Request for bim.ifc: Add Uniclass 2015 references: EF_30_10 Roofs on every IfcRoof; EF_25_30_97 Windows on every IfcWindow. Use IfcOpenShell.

First a look at what the model holds.

```python
import ifcopenshell

model = ifcopenshell.open("bim.ifc")
print(model.schema)
print("classifications:", [c.Name for c in model.by_type("IfcClassification")])
for ifc_class in ("IfcDoor", "IfcRoof", "IfcStair", "IfcWall", "IfcWindow"):
    print(ifc_class, len(model.by_type(ifc_class)))
```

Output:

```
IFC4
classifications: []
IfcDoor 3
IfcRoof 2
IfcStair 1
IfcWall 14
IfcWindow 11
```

```python
import ifcopenshell
import ifcopenshell.api.classification

model = ifcopenshell.open("bim.ifc")

system = ifcopenshell.api.classification.add_classification(model, classification="Uniclass 2015")

codes = {
    "IfcRoof": ("EF_30_10", "Roofs"),
    "IfcWindow": ("EF_25_30_97", "Windows"),
}
for ifc_class, (code, name) in codes.items():
    products = model.by_type(ifc_class)
    ifcopenshell.api.classification.add_reference(
        model, products=products, classification=system, identification=code, name=name
    )
    print(code, len(products))

model.write("bim_updated.ifc")
```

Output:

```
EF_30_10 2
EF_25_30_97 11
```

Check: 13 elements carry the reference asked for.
